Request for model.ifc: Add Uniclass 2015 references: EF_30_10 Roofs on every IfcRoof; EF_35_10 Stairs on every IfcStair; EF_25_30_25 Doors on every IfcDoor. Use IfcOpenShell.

First a look at what the model holds.

```python
import ifcopenshell

model = ifcopenshell.open("model.ifc")
print(model.schema)
print("classifications:", [c.Name for c in model.by_type("IfcClassification")])
for ifc_class in ("IfcDoor", "IfcRoof", "IfcStair", "IfcWall", "IfcWindow"):
    print(ifc_class, len(model.by_type(ifc_class)))
```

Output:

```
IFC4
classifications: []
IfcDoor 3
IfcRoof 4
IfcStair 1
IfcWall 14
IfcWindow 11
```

```python
import ifcopenshell
import ifcopenshell.api.classification

model = ifcopenshell.open("model.ifc")

system = ifcopenshell.api.classification.add_classification(model, classification="Uniclass 2015")

codes = {
    "IfcRoof": ("EF_30_10", "Roofs"),
    "IfcStair": ("EF_35_10", "Stairs"),
    "IfcDoor": ("EF_25_30_25", "Doors"),
}
for ifc_class, (code, name) in codes.items():
    products = model.by_type(ifc_class)
    ifcopenshell.api.classification.add_reference(
        model, products=products, classification=system, identification=code, name=name
    )
    print(code, len(products))

model.write("model_v2.ifc")
```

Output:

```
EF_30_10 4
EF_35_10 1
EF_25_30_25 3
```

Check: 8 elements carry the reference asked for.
